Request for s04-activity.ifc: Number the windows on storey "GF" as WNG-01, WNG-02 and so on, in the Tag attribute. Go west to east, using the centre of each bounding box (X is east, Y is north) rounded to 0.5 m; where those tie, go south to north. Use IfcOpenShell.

First a look at what the model holds.

```python
import ifcopenshell
import ifcopenshell.util.element
import ifcopenshell.util.placement

model = ifcopenshell.open("s04-activity.ifc")
print(model.schema)
storey = next(s for s in model.by_type("IfcBuildingStorey") if s.Name == "GF")
windows = [e for e in ifcopenshell.util.element.get_decomposition(storey) if e.is_a("IfcWindow")]
for e in sorted(windows, key=lambda e: e.id()):
    origin = ifcopenshell.util.placement.get_local_placement(e.ObjectPlacement)[:3, 3]
    print(e.id(), e.Tag, e.Name, origin.round(2) + 0.0, sep=" | ")
```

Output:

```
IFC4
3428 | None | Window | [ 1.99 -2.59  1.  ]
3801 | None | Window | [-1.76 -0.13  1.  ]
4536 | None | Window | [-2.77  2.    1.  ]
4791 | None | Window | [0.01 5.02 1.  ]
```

```python
import ifcopenshell
import ifcopenshell.geom
import ifcopenshell.util.element
import ifcopenshell.util.shape

model = ifcopenshell.open("s04-activity.ifc")
settings = ifcopenshell.geom.settings()
settings.set("use-world-coords", True)


def centre(element):
    shape = ifcopenshell.geom.create_shape(settings, element)
    return ifcopenshell.util.shape.get_bbox_centroid(shape.geometry)


storey = next(s for s in model.by_type("IfcBuildingStorey") if s.Name == "GF")
windows = [e for e in ifcopenshell.util.element.get_decomposition(storey) if e.is_a("IfcWindow")]

# Insertion points can sit at a corner or the storey origin, so sort by the geometry (in metres).
centres = {e: centre(e) for e in windows}
windows.sort(key=lambda e: (round(centres[e][0] / 0.5), centres[e][1]))

for i, e in enumerate(windows, start=1):
    number = f"WNG-{i:02d}"
    e.Tag = number
    print(e.id(), number)

model.write("s04-activity-out.ifc")
```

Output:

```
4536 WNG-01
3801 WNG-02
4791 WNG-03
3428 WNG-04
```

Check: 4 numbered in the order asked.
